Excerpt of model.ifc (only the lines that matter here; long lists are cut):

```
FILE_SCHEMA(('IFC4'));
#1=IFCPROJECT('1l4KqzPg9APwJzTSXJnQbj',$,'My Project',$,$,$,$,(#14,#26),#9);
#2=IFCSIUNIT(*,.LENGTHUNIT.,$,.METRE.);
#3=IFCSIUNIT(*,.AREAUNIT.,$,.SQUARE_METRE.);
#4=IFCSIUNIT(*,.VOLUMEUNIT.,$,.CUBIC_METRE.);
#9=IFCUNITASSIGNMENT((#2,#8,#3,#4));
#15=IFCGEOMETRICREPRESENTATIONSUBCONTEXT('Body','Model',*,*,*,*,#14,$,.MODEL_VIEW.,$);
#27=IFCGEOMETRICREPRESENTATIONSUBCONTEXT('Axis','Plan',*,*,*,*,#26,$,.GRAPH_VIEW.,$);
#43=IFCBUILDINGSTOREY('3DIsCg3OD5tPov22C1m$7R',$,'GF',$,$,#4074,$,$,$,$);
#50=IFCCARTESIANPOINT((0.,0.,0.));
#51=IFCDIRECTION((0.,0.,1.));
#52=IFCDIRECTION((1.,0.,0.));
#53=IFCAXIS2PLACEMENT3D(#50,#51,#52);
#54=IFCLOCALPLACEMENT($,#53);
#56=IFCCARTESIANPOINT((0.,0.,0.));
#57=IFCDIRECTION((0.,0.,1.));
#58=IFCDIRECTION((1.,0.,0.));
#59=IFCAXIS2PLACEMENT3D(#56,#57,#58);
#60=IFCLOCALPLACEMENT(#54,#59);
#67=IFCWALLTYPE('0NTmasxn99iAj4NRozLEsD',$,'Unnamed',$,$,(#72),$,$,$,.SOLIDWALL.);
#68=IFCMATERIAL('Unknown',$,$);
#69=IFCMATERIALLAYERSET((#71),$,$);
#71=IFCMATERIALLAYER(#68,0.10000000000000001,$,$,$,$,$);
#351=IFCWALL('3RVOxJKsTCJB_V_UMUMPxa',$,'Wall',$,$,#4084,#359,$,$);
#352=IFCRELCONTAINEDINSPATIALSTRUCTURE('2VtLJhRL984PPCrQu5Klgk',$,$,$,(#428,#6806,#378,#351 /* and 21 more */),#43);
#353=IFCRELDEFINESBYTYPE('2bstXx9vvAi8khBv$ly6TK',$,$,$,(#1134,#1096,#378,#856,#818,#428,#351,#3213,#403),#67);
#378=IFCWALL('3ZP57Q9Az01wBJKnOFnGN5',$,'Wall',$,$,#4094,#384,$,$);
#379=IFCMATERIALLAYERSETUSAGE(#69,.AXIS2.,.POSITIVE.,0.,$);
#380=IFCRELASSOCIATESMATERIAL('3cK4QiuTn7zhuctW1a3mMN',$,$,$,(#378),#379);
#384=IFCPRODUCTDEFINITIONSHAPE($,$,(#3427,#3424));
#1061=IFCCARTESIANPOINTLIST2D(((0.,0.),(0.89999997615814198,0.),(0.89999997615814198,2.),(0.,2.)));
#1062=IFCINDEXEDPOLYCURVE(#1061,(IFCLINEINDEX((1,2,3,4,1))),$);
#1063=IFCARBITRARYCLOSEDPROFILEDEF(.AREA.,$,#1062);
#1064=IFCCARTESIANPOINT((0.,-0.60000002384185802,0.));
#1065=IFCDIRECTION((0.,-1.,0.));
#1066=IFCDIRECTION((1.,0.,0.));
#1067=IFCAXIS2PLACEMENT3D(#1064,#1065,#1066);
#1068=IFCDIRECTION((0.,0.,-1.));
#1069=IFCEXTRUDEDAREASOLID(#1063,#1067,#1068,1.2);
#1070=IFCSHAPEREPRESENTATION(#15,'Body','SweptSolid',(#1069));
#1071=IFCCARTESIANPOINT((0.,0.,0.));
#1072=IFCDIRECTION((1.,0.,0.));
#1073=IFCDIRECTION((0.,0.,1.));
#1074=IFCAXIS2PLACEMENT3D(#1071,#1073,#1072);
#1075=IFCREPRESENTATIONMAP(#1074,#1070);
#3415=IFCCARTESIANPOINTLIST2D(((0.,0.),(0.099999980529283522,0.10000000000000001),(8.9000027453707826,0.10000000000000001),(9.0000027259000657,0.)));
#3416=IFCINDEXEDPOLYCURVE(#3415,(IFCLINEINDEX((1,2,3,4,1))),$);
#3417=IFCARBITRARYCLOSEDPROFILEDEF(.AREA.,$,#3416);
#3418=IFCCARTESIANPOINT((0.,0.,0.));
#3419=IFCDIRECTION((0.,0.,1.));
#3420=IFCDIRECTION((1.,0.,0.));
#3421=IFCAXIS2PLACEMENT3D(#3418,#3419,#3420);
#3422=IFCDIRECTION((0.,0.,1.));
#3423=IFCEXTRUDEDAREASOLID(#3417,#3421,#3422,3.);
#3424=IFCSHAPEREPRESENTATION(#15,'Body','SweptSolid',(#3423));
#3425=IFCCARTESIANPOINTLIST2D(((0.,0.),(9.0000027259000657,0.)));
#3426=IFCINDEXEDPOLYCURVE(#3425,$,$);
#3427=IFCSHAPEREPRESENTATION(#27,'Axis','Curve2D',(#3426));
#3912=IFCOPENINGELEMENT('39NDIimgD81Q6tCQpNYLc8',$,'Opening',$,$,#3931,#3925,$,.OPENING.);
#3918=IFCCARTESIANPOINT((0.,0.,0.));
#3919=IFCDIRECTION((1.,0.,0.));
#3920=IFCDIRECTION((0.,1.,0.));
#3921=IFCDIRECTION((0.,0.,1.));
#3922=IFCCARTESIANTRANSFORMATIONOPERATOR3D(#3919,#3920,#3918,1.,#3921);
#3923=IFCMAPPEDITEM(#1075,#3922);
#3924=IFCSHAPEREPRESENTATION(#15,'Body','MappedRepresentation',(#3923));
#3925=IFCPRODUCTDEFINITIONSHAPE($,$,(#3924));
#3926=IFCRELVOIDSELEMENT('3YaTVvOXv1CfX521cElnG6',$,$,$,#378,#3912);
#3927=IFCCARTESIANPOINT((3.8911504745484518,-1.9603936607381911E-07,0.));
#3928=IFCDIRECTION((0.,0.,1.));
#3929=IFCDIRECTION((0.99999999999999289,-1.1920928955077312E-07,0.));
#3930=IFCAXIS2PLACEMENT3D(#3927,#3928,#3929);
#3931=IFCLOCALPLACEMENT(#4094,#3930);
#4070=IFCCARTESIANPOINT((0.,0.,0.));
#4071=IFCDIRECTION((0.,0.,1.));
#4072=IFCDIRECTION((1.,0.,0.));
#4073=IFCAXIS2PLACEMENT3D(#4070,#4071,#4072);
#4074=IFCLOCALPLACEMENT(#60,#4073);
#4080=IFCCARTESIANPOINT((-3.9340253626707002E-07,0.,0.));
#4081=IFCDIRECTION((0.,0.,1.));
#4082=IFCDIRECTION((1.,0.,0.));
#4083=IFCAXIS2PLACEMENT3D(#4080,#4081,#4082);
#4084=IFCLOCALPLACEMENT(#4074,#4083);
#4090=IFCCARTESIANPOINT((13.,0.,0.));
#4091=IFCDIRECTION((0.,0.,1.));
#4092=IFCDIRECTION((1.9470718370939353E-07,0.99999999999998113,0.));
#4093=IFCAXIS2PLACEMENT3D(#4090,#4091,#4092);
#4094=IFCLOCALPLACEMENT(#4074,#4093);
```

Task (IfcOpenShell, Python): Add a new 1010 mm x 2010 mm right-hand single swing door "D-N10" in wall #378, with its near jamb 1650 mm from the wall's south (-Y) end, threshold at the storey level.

```python
import numpy as np
import ifcopenshell
import ifcopenshell.api.feature
import ifcopenshell.api.geometry
import ifcopenshell.api.root
import ifcopenshell.api.spatial
import ifcopenshell.geom
import ifcopenshell.util.element
import ifcopenshell.util.placement
import ifcopenshell.util.representation
import ifcopenshell.util.shape
import ifcopenshell.util.unit

model = ifcopenshell.open("model.ifc")
unit_scale = ifcopenshell.util.unit.calculate_unit_scale(model)
settings = ifcopenshell.geom.settings()


def volume(element):
    """Net volume in cubic metres, openings subtracted."""
    shape = ifcopenshell.geom.create_shape(settings, element)
    return ifcopenshell.util.shape.get_volume(shape.geometry)


wall = model.by_guid("3ZP57Q9Az01wBJKnOFnGN5")
storey = ifcopenshell.util.element.get_container(wall, ifc_class="IfcBuildingStorey")
context = ifcopenshell.util.representation.get_context(model, "Model", "Body", "MODEL_VIEW")
before = volume(wall)

width, height, from_end, sill = 1.01, 2.01, 1.65, 0.0  # metres

# The wall runs along its own X axis, and the end named is its -X end.
wall_shape = ifcopenshell.geom.create_shape(settings, wall)
x, y, z = ifcopenshell.util.shape.get_vertices(wall_shape.geometry).T
start = x.min() + from_end
face, thickness = float(y.min()), float(y.max() - y.min())
wall_matrix = ifcopenshell.util.placement.get_local_placement(wall.ObjectPlacement)
level = ifcopenshell.util.placement.get_local_placement(storey.ObjectPlacement)[2, 3]


def in_wall(x, y):
    """Placement at x, y metres in the wall's axes, at sill height."""
    matrix = wall_matrix.copy()
    matrix[:, 3] = wall_matrix @ np.array([x / unit_scale, y / unit_scale, 0.0, 1.0])
    matrix[2, 3] = level + sill / unit_scale
    return matrix


# Opening: a box that overshoots both wall faces by 50 mm.
opening = ifcopenshell.api.root.create_entity(model, ifc_class="IfcOpeningElement", predefined_type="OPENING")
box = ifcopenshell.api.geometry.add_wall_representation(
    model, context=context, length=width, height=height, thickness=thickness + 0.1
)
ifcopenshell.api.geometry.assign_representation(model, product=opening, representation=box)
ifcopenshell.api.geometry.edit_object_placement(model, product=opening, matrix=in_wall(start, face - 0.05), is_si=False)
ifcopenshell.api.feature.add_feature(model, feature=opening, element=wall)

door = ifcopenshell.api.root.create_entity(model, ifc_class="IfcDoor", name="D-N10", predefined_type="DOOR")
door.OverallWidth, door.OverallHeight = width / unit_scale, height / unit_scale
door.OperationType = "SINGLE_SWING_RIGHT"
body = ifcopenshell.api.geometry.add_door_representation(
    model,
    context=context,
    overall_width=door.OverallWidth,
    overall_height=door.OverallHeight,
    operation_type="SINGLE_SWING_RIGHT",
    lining_properties={"LiningDepth": thickness / unit_scale, "ThresholdDepth": thickness / unit_scale},
)
ifcopenshell.api.geometry.assign_representation(model, product=door, representation=body)
ifcopenshell.api.spatial.assign_container(model, products=[door], relating_structure=storey)
ifcopenshell.api.feature.add_filling(model, opening=opening, element=door)

# The lining spans the wall, so the door starts at the wall face.
ifcopenshell.api.geometry.edit_object_placement(model, product=door, matrix=in_wall(start, face), is_si=False)

after = volume(wall)

print(f"wall volume {before:.3f} -> {after:.3f} m3")

model.write("model-out.ifc")
```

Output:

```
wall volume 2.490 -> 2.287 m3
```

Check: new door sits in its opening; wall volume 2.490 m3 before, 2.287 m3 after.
